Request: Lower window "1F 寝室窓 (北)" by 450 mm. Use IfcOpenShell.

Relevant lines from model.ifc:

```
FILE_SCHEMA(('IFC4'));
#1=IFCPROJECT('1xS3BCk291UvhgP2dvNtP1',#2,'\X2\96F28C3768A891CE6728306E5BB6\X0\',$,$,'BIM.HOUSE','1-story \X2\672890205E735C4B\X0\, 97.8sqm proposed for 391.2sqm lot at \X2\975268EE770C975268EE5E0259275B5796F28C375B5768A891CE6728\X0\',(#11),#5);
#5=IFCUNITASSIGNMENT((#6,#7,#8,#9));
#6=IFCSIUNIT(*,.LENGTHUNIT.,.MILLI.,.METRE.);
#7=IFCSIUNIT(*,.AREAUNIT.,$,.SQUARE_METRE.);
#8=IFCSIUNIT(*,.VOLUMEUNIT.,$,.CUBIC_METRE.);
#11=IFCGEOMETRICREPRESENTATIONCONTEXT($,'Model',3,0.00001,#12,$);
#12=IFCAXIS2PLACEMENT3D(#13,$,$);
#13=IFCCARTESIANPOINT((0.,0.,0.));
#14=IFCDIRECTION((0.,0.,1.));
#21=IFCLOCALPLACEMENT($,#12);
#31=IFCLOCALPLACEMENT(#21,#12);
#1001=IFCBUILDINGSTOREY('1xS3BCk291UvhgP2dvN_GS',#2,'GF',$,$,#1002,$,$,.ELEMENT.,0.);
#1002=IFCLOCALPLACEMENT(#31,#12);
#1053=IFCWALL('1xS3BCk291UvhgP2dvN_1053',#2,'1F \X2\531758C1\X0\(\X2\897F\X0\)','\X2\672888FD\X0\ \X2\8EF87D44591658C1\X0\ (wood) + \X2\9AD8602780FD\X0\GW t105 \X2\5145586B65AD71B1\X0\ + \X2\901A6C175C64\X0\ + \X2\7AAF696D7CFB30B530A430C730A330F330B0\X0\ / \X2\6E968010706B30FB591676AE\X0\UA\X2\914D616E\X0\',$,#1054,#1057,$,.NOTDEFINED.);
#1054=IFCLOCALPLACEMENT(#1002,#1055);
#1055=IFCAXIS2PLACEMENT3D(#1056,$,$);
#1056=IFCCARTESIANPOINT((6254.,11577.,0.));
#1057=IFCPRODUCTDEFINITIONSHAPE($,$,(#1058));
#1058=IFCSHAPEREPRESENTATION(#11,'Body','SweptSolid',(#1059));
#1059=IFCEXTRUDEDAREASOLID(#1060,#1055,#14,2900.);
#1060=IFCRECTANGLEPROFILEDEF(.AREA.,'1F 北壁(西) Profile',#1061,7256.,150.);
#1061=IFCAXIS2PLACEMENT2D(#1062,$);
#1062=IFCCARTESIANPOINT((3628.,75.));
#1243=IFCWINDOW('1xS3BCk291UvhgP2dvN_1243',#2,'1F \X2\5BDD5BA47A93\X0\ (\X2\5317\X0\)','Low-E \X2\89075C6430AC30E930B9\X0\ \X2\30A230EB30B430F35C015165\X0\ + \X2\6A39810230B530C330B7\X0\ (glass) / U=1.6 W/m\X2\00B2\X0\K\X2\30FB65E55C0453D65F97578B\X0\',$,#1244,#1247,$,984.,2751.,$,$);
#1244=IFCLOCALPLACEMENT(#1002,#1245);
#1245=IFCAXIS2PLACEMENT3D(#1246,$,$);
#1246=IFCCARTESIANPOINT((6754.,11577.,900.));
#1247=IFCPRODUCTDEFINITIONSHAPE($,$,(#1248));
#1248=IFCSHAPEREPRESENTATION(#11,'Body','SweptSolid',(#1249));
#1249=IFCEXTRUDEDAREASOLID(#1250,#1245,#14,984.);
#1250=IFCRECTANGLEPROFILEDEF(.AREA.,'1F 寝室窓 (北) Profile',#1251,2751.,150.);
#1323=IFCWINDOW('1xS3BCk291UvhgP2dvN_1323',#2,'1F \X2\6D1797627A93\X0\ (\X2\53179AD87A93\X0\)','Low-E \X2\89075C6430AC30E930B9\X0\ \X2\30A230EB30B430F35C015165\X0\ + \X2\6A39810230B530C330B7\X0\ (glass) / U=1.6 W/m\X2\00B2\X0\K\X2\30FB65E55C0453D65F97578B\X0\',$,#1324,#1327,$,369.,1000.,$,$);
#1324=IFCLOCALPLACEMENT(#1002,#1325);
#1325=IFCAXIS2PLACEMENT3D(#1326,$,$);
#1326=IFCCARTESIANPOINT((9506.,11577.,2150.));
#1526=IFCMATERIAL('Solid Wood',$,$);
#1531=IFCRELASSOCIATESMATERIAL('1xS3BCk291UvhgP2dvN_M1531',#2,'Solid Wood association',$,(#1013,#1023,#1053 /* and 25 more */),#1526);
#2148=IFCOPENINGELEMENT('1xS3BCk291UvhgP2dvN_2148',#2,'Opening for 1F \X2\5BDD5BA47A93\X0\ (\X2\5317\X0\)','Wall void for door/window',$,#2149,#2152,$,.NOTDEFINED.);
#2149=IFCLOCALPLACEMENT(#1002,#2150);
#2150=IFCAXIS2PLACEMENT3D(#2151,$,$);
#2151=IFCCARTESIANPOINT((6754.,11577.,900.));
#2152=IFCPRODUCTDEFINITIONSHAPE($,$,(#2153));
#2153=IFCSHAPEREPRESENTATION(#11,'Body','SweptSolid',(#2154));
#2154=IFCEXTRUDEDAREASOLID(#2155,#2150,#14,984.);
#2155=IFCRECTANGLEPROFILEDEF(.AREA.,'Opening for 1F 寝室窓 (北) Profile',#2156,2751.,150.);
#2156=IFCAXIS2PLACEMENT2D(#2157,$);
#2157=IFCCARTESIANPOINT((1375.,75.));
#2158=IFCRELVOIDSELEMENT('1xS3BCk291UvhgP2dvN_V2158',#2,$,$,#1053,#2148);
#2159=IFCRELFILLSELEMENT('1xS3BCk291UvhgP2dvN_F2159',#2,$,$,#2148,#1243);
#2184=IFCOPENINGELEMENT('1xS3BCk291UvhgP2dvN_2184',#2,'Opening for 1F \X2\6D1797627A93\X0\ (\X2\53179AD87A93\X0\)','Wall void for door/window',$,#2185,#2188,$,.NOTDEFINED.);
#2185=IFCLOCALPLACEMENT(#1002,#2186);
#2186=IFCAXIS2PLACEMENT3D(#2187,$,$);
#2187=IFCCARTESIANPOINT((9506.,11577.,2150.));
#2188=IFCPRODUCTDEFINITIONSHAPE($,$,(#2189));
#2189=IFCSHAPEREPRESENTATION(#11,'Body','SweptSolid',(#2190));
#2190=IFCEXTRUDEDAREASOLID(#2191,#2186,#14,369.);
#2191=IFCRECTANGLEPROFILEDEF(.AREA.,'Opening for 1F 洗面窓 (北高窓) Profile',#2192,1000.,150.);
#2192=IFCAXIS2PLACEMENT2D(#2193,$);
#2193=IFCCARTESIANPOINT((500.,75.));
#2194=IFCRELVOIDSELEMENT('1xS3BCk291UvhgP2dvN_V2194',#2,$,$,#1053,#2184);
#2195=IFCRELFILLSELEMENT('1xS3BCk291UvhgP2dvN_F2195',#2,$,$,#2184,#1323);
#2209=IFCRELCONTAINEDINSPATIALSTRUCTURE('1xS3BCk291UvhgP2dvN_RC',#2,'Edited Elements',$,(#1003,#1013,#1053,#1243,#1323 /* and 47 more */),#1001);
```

```python
import numpy as np
import ifcopenshell
import ifcopenshell.api.geometry
import ifcopenshell.util.placement
import ifcopenshell.util.unit

model = ifcopenshell.open("model.ifc")
unit_scale = ifcopenshell.util.unit.calculate_unit_scale(model)

window = model.by_guid("1xS3BCk291UvhgP2dvN_1243")
opening = window.FillsVoids[0].RelatingOpeningElement
dz = -0.45 / unit_scale

shift = np.array([0.0, 0.0, dz])
# The window is not placed relative to its opening, so move both.
for product in (opening, window):
    matrix = ifcopenshell.util.placement.get_local_placement(product.ObjectPlacement)
    matrix[:3, 3] += shift
    ifcopenshell.api.geometry.edit_object_placement(model, product=product, matrix=matrix, is_si=False)

print(f"moved by {dz * unit_scale:+.3f} m")

model.write("model_v2.ifc")
```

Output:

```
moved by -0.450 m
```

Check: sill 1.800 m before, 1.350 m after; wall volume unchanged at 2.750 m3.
